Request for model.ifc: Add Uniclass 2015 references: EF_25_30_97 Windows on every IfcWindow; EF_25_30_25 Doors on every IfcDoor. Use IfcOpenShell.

First a look at what the model holds.

```python
import ifcopenshell

model = ifcopenshell.open("model.ifc")
print(model.schema)
print("classifications:", [c.Name for c in model.by_type("IfcClassification")])
for ifc_class in ("IfcDoor", "IfcRoof", "IfcStair", "IfcWall", "IfcWindow"):
    print(ifc_class, len(model.by_type(ifc_class)))
```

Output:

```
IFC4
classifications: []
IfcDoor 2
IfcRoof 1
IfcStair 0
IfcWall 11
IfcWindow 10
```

```python
import ifcopenshell
import ifcopenshell.api.classification

model = ifcopenshell.open("model.ifc")

system = ifcopenshell.api.classification.add_classification(model, classification="Uniclass 2015")

codes = {
    "IfcWindow": ("EF_25_30_97", "Windows"),
    "IfcDoor": ("EF_25_30_25", "Doors"),
}
for ifc_class, (code, name) in codes.items():
    products = model.by_type(ifc_class)
    ifcopenshell.api.classification.add_reference(
        model, products=products, classification=system, identification=code, name=name
    )
    print(code, len(products))

model.write("model_v2.ifc")
```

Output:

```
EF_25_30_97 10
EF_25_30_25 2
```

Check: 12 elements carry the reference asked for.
